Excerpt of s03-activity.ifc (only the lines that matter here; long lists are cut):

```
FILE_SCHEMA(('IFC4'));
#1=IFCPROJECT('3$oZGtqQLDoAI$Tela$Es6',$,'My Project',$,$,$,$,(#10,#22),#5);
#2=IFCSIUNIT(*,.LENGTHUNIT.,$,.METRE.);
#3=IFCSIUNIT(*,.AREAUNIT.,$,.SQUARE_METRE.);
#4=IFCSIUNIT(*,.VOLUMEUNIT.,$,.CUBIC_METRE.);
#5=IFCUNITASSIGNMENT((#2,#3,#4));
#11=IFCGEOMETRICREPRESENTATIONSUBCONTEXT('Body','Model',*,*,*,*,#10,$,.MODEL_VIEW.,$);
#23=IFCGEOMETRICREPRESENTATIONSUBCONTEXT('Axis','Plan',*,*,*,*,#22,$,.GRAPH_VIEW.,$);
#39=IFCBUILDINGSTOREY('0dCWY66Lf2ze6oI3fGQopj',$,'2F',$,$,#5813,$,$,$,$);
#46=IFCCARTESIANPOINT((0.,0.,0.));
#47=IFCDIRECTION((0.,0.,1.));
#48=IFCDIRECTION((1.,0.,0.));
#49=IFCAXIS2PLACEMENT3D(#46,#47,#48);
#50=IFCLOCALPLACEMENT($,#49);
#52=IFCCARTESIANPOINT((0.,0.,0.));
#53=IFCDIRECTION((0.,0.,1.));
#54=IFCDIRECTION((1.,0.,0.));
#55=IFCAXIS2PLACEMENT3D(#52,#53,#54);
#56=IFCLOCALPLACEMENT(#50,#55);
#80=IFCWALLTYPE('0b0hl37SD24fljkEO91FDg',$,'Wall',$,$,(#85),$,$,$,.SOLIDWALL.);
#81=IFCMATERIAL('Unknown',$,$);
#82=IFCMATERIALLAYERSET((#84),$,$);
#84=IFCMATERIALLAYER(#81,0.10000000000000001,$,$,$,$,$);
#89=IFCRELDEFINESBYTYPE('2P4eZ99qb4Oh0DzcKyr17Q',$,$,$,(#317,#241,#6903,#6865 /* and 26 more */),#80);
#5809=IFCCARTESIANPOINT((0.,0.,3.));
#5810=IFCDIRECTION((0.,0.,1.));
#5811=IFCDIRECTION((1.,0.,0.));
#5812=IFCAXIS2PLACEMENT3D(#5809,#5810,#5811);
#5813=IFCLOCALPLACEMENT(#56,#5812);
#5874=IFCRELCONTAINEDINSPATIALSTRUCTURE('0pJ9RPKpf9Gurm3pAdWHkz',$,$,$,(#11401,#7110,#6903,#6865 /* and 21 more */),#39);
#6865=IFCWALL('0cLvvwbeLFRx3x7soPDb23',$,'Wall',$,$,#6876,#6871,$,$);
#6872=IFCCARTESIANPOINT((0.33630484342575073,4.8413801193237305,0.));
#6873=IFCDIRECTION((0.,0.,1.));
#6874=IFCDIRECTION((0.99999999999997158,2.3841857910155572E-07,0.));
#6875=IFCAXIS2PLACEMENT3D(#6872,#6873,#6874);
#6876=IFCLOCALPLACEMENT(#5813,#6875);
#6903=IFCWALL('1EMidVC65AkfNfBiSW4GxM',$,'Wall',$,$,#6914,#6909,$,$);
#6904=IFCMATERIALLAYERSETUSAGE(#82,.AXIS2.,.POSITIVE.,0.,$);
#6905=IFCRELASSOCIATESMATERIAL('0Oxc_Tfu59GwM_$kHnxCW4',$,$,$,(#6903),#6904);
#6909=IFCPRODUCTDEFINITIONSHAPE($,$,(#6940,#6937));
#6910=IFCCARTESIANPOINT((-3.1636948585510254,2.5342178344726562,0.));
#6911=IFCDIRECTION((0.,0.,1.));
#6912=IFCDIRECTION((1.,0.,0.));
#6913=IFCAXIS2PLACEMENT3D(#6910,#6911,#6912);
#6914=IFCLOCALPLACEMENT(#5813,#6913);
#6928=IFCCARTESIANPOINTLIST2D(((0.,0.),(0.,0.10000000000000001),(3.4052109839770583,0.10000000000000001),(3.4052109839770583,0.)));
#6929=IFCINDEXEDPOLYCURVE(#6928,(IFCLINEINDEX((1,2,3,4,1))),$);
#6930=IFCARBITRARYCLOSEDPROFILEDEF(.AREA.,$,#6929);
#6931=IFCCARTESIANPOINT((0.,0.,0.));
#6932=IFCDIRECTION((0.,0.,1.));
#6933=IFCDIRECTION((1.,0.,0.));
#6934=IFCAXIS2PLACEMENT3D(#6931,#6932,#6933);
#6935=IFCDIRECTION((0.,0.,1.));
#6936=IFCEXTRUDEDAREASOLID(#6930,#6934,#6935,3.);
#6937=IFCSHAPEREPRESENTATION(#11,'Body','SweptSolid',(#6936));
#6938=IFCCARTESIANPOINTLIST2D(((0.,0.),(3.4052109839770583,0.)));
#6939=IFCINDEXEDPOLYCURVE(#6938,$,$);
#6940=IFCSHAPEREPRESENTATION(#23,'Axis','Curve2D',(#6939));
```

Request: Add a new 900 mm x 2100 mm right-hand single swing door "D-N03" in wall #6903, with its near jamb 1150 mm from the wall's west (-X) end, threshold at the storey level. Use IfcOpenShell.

```python
import numpy as np
import ifcopenshell
import ifcopenshell.api.feature
import ifcopenshell.api.geometry
import ifcopenshell.api.root
import ifcopenshell.api.spatial
import ifcopenshell.geom
import ifcopenshell.util.element
import ifcopenshell.util.placement
import ifcopenshell.util.representation
import ifcopenshell.util.shape
import ifcopenshell.util.unit

model = ifcopenshell.open("s03-activity.ifc")
unit_scale = ifcopenshell.util.unit.calculate_unit_scale(model)
settings = ifcopenshell.geom.settings()


def volume(element):
    """Net volume in cubic metres, openings subtracted."""
    shape = ifcopenshell.geom.create_shape(settings, element)
    return ifcopenshell.util.shape.get_volume(shape.geometry)


wall = model.by_guid("1EMidVC65AkfNfBiSW4GxM")
storey = ifcopenshell.util.element.get_container(wall, ifc_class="IfcBuildingStorey")
context = ifcopenshell.util.representation.get_context(model, "Model", "Body", "MODEL_VIEW")
before = volume(wall)

width, height, from_end, sill = 0.9, 2.1, 1.15, 0.0  # metres

# The wall runs along its own X axis, and the end named is its -X end.
wall_shape = ifcopenshell.geom.create_shape(settings, wall)
x, y, z = ifcopenshell.util.shape.get_vertices(wall_shape.geometry).T
start = x.min() + from_end
face, thickness = float(y.min()), float(y.max() - y.min())
wall_matrix = ifcopenshell.util.placement.get_local_placement(wall.ObjectPlacement)
level = ifcopenshell.util.placement.get_local_placement(storey.ObjectPlacement)[2, 3]


def in_wall(x, y):
    """Placement at x, y metres in the wall's axes, at sill height."""
    matrix = wall_matrix.copy()
    matrix[:, 3] = wall_matrix @ np.array([x / unit_scale, y / unit_scale, 0.0, 1.0])
    matrix[2, 3] = level + sill / unit_scale
    return matrix


# Opening: a box that overshoots both wall faces by 50 mm.
opening = ifcopenshell.api.root.create_entity(model, ifc_class="IfcOpeningElement", predefined_type="OPENING")
box = ifcopenshell.api.geometry.add_wall_representation(
    model, context=context, length=width, height=height, thickness=thickness + 0.1
)
ifcopenshell.api.geometry.assign_representation(model, product=opening, representation=box)
ifcopenshell.api.geometry.edit_object_placement(model, product=opening, matrix=in_wall(start, face - 0.05), is_si=False)
ifcopenshell.api.feature.add_feature(model, feature=opening, element=wall)

door = ifcopenshell.api.root.create_entity(model, ifc_class="IfcDoor", name="D-N03", predefined_type="DOOR")
door.OverallWidth, door.OverallHeight = width / unit_scale, height / unit_scale
door.OperationType = "SINGLE_SWING_RIGHT"
body = ifcopenshell.api.geometry.add_door_representation(
    model,
    context=context,
    overall_width=door.OverallWidth,
    overall_height=door.OverallHeight,
    operation_type="SINGLE_SWING_RIGHT",
    lining_properties={"LiningDepth": thickness / unit_scale, "ThresholdDepth": thickness / unit_scale},
)
ifcopenshell.api.geometry.assign_representation(model, product=door, representation=body)
ifcopenshell.api.spatial.assign_container(model, products=[door], relating_structure=storey)
ifcopenshell.api.feature.add_filling(model, opening=opening, element=door)

# The lining spans the wall, so the door starts at the wall face.
ifcopenshell.api.geometry.edit_object_placement(model, product=door, matrix=in_wall(start, face), is_si=False)

after = volume(wall)

print(f"wall volume {before:.3f} -> {after:.3f} m3")

model.write("s03-activity_rev.ifc")
```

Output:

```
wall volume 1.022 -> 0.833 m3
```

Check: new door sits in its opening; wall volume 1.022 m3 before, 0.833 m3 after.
